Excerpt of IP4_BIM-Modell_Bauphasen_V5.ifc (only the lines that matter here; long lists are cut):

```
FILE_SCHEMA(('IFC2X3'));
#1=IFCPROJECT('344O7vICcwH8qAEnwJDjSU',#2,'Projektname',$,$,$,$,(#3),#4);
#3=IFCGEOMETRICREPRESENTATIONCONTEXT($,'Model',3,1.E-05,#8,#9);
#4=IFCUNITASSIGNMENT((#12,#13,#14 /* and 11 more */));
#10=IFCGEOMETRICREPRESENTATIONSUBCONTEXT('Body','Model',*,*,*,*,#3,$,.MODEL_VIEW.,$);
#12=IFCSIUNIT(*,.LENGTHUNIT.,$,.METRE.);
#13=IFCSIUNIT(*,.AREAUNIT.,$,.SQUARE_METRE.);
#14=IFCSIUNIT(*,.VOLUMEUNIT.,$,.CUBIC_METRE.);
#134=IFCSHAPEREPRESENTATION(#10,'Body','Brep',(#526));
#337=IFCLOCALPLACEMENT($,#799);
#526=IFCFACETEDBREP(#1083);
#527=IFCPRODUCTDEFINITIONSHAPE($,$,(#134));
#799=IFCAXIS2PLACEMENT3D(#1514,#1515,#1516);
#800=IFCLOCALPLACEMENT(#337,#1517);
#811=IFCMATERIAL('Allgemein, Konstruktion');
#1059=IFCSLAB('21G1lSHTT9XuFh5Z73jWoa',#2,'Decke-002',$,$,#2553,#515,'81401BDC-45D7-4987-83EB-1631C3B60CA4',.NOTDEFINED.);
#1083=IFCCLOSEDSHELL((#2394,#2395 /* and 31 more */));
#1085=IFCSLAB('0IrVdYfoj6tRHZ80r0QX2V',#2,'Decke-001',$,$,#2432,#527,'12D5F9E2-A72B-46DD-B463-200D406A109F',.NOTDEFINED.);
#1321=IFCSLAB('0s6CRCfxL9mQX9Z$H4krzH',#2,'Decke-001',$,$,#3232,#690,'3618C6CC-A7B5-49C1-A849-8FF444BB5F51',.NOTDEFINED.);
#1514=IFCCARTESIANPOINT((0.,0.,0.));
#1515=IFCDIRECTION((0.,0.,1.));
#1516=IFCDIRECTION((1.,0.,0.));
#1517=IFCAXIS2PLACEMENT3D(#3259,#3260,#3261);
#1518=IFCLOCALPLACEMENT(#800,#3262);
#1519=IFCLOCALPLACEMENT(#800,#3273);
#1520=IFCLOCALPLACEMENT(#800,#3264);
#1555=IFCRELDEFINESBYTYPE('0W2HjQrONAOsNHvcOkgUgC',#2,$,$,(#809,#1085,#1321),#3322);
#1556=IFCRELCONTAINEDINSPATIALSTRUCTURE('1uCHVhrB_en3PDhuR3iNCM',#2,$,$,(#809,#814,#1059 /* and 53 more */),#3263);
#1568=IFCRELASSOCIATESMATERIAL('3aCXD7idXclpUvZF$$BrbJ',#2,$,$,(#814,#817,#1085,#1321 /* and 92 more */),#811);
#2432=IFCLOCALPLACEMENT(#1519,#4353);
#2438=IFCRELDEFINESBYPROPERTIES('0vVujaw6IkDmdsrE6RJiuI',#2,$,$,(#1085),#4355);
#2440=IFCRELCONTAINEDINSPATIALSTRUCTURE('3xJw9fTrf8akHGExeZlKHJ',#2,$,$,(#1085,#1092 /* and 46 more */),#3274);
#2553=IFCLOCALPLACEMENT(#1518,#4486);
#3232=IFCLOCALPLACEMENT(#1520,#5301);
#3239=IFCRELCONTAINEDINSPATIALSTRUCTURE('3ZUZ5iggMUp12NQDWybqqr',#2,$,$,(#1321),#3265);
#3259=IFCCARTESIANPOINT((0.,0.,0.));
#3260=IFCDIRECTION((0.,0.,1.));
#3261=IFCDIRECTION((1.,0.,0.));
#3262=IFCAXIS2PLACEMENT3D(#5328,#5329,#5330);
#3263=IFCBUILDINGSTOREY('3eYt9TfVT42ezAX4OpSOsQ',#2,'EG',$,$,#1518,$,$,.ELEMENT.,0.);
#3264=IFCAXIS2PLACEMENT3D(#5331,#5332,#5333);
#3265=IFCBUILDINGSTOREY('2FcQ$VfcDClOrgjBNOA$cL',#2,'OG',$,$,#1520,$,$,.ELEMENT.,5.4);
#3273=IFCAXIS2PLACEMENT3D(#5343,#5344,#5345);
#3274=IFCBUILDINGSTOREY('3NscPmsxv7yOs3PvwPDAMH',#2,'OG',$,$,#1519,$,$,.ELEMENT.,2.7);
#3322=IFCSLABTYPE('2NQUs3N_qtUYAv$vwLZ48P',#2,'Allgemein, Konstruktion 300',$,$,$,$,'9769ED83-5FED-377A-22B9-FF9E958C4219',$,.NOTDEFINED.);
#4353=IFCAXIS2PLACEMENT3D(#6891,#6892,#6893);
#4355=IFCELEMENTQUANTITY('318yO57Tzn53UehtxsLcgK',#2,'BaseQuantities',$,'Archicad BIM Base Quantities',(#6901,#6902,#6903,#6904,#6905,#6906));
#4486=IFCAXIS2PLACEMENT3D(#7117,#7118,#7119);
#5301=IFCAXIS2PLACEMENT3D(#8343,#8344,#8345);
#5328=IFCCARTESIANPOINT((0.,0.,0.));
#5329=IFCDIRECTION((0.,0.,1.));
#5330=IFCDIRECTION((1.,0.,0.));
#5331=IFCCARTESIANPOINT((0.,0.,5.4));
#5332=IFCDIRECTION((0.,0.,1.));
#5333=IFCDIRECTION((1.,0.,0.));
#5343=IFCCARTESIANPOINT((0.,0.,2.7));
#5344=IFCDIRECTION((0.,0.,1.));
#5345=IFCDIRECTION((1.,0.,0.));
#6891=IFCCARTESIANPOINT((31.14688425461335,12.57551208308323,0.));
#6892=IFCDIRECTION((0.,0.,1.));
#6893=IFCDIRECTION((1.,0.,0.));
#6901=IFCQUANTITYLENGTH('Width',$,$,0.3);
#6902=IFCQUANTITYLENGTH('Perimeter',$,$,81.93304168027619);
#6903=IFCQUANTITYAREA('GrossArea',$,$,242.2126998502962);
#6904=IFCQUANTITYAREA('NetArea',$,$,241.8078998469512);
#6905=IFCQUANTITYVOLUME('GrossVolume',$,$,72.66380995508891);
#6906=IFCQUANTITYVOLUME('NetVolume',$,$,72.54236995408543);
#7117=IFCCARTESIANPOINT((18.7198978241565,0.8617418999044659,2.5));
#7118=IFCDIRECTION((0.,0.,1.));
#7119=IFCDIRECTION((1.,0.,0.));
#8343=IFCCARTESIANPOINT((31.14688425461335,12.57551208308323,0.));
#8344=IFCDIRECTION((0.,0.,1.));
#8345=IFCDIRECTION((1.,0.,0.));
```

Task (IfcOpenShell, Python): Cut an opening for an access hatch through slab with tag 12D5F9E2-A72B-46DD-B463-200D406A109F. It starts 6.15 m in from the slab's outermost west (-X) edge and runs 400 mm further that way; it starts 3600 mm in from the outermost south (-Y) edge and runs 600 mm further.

```python
import numpy as np
import ifcopenshell
import ifcopenshell.api.feature
import ifcopenshell.api.geometry
import ifcopenshell.api.pset
import ifcopenshell.api.root
import ifcopenshell.geom
import ifcopenshell.util.element
import ifcopenshell.util.placement
import ifcopenshell.util.representation
import ifcopenshell.util.shape
import ifcopenshell.util.unit

model = ifcopenshell.open("IP4_BIM-Modell_Bauphasen_V5.ifc")
unit_scale = ifcopenshell.util.unit.calculate_unit_scale(model)
area_scale = ifcopenshell.util.unit.calculate_unit_scale(model, "AREAUNIT")
volume_scale = ifcopenshell.util.unit.calculate_unit_scale(model, "VOLUMEUNIT")
settings = ifcopenshell.geom.settings()


def volume(element):
    """Net volume in cubic metres, openings subtracted."""
    shape = ifcopenshell.geom.create_shape(settings, element)
    return ifcopenshell.util.shape.get_volume(shape.geometry)


slab = model.by_id(1085)
before = volume(slab)

# Extent in the slab's own axes, in metres. The edges named are its -X and -Y sides.
slab_shape = ifcopenshell.geom.create_shape(settings, slab)
vertices = ifcopenshell.util.shape.get_vertices(slab_shape.geometry)
x_min, y_min, bottom = vertices.min(axis=0)
top = vertices[:, 2].max()

opening = ifcopenshell.api.root.create_entity(model, ifc_class="IfcOpeningElement", name="Access hatch opening")
context = ifcopenshell.util.representation.get_context(model, "Model", "Body", "MODEL_VIEW")
width, depth = 0.4, 0.6
outline = [(0.0, 0.0), (width, 0.0), (width, depth), (0.0, depth), (0.0, 0.0)]
# Overshoot both faces by 50 mm so the cut is clean.
shape = ifcopenshell.api.geometry.add_slab_representation(
    model, context=context, depth=top - bottom + 0.1, polyline=outline
)
ifcopenshell.api.geometry.assign_representation(model, product=opening, representation=shape)

matrix = ifcopenshell.util.placement.get_local_placement(slab.ObjectPlacement)
matrix[:, 3] = matrix @ np.append(np.array([x_min + 6.15, y_min + 3.6, bottom - 0.05]) / unit_scale, 1.0)
ifcopenshell.api.geometry.edit_object_placement(model, product=opening, matrix=matrix, is_si=False)
ifcopenshell.api.feature.add_feature(model, feature=opening, element=slab)

after = volume(slab)

# Update the slab's stored quantities.
qto = model.by_id(ifcopenshell.util.element.get_pset(slab, "BaseQuantities", should_inherit=False)["id"])
ifcopenshell.api.pset.edit_qto(model, qto=qto, properties={
    "NetArea": after / (top - bottom) / area_scale,
    "NetVolume": after / volume_scale,
})

print(f"slab volume {before:.3f} -> {after:.3f} m3")

model.write("IP4_BIM-Modell_Bauphasen_V5-out.ifc")
```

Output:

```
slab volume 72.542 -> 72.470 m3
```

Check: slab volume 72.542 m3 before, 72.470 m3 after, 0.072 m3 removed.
